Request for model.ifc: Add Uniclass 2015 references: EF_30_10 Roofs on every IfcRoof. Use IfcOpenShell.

First a look at what the model holds.

```python
import ifcopenshell

model = ifcopenshell.open("model.ifc")
print(model.schema)
print("classifications:", [c.Name for c in model.by_type("IfcClassification")])
for ifc_class in ("IfcDoor", "IfcRoof", "IfcStair", "IfcWall", "IfcWindow"):
    print(ifc_class, len(model.by_type(ifc_class)))
```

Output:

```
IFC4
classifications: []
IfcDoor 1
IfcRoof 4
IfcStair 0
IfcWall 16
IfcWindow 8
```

```python
import ifcopenshell
import ifcopenshell.api.classification

model = ifcopenshell.open("model.ifc")

system = ifcopenshell.api.classification.add_classification(model, classification="Uniclass 2015")

codes = {
    "IfcRoof": ("EF_30_10", "Roofs"),
}
for ifc_class, (code, name) in codes.items():
    products = model.by_type(ifc_class)
    ifcopenshell.api.classification.add_reference(
        model, products=products, classification=system, identification=code, name=name
    )
    print(code, len(products))

model.write("model-out.ifc")
```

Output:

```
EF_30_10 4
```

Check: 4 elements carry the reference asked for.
